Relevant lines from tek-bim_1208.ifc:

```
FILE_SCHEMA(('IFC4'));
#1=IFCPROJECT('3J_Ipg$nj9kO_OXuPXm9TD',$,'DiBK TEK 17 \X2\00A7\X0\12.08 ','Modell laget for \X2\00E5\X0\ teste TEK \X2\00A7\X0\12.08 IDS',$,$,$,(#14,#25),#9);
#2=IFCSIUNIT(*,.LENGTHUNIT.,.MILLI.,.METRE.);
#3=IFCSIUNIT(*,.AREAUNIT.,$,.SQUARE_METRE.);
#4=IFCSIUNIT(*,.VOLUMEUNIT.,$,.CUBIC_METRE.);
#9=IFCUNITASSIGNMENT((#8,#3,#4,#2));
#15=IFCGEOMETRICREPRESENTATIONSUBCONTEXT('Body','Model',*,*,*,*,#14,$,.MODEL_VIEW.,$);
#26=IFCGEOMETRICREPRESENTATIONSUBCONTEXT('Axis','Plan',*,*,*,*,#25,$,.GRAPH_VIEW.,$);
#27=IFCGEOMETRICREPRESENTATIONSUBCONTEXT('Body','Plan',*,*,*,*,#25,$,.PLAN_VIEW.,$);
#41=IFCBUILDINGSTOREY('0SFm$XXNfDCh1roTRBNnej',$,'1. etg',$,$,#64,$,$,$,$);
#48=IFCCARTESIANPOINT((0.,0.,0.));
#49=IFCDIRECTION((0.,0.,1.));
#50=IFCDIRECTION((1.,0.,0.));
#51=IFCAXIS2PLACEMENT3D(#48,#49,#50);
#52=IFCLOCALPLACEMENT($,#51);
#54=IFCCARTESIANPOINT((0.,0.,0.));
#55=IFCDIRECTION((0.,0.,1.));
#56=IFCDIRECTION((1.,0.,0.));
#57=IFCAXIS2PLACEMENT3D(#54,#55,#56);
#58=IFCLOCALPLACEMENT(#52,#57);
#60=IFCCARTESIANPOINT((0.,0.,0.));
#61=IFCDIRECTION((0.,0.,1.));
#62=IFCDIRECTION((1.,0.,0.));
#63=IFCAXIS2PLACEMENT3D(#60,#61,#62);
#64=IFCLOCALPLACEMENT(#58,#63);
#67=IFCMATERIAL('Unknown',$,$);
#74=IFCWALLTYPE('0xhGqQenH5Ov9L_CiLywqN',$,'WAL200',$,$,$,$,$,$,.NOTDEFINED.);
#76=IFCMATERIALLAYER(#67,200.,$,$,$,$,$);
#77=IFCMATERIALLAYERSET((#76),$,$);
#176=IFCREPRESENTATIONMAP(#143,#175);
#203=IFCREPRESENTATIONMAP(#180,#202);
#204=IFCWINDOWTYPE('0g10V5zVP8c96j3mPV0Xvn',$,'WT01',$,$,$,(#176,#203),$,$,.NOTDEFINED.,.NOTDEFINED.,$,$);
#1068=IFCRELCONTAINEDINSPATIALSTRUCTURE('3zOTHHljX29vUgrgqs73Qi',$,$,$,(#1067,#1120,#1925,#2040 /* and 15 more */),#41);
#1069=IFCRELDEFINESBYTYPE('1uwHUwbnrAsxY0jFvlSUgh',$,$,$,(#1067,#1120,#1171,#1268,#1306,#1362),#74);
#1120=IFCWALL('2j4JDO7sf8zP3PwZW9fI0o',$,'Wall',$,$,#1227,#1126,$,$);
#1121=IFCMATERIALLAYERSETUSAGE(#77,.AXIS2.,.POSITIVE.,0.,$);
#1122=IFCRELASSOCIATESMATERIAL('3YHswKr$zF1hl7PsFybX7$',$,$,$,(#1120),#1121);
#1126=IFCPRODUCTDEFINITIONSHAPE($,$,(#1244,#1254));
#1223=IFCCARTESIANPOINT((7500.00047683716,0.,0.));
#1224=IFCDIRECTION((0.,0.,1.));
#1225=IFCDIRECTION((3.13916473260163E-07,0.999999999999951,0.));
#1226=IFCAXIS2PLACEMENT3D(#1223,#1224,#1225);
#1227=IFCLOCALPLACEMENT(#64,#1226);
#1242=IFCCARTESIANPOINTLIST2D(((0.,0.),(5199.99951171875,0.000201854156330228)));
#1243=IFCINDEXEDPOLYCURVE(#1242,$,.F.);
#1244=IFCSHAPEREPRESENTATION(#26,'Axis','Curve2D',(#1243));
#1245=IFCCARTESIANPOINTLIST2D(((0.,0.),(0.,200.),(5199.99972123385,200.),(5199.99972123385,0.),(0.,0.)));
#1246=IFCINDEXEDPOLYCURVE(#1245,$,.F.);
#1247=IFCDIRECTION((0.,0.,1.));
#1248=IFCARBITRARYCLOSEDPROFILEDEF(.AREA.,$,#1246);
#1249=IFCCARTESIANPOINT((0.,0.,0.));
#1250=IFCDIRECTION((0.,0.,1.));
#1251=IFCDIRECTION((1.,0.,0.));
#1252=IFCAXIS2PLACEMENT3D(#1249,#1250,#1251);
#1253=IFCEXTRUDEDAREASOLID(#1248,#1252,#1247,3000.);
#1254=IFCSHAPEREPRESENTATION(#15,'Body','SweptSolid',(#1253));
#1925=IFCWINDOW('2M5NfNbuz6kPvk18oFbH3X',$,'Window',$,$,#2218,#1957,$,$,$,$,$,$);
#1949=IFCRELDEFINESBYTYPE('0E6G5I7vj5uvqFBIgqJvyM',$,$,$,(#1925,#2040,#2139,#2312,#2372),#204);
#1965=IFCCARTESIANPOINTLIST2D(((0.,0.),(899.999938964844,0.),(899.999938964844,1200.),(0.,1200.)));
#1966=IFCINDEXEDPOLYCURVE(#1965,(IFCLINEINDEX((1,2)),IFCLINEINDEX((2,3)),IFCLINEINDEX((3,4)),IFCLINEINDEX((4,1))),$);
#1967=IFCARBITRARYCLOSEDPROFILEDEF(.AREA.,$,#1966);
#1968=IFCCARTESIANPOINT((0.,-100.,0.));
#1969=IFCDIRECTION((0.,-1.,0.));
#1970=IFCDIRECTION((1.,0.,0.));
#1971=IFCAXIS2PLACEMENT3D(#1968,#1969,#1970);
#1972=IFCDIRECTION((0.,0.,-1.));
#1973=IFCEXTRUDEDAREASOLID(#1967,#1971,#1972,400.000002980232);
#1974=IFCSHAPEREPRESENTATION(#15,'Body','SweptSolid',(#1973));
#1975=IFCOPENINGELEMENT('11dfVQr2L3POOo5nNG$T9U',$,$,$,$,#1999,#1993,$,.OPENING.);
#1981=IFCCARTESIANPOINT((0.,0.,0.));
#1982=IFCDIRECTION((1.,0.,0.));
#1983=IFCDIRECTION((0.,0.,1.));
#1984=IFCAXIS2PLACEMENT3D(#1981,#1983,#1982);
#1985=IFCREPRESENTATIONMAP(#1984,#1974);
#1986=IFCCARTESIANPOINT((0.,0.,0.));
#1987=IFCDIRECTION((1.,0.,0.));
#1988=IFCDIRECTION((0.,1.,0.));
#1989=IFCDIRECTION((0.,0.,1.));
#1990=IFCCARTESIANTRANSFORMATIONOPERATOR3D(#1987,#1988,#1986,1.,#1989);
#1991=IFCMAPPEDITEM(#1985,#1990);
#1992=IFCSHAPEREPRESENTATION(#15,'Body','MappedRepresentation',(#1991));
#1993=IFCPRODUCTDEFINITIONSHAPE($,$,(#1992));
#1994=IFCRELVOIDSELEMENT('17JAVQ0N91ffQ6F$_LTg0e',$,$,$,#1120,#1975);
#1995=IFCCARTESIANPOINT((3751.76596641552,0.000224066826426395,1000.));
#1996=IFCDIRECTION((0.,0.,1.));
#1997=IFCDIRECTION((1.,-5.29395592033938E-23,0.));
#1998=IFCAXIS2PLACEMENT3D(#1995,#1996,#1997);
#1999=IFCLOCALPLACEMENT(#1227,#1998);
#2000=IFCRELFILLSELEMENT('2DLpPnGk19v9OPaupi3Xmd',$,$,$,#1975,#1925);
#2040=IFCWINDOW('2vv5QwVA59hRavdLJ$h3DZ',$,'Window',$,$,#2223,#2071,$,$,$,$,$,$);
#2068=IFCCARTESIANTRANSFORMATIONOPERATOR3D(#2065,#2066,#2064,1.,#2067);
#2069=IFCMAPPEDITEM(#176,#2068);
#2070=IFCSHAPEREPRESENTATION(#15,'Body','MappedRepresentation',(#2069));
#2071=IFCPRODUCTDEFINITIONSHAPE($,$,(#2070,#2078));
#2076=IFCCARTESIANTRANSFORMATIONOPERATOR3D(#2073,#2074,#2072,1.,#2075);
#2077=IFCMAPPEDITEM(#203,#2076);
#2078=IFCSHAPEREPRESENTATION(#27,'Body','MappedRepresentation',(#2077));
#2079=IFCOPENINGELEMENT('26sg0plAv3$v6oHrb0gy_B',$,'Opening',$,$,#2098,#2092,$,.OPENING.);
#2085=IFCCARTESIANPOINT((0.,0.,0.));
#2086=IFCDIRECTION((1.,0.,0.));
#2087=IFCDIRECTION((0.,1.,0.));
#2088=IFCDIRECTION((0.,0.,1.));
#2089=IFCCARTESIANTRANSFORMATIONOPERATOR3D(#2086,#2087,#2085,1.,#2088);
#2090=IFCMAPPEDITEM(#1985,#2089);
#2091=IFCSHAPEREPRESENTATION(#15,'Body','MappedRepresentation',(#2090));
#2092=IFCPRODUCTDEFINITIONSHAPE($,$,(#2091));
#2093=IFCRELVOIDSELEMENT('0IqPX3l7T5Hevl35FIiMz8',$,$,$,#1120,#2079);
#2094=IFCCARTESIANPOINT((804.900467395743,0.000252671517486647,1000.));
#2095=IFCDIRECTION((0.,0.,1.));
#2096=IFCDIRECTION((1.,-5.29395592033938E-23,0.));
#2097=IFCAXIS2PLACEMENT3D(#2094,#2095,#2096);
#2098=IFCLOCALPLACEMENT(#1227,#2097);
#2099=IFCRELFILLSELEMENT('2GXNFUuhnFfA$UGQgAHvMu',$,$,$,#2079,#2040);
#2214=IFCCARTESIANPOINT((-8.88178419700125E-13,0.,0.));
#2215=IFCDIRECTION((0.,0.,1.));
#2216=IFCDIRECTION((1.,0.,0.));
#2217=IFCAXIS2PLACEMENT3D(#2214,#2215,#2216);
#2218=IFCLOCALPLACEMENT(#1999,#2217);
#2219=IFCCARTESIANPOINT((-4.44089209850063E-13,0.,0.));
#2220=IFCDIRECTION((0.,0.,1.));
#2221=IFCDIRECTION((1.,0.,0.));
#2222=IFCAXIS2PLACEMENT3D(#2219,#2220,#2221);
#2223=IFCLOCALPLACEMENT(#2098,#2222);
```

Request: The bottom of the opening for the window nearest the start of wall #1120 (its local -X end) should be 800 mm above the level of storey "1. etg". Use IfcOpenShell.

```python
import numpy as np
import ifcopenshell
import ifcopenshell.api.geometry
import ifcopenshell.geom
import ifcopenshell.util.element
import ifcopenshell.util.placement
import ifcopenshell.util.shape
import ifcopenshell.util.unit

model = ifcopenshell.open("tek-bim_1208.ifc")
unit_scale = ifcopenshell.util.unit.calculate_unit_scale(model)

window = model.by_id(2040)
opening = window.FillsVoids[0].RelatingOpeningElement
storey = ifcopenshell.util.element.get_container(window, ifc_class="IfcBuildingStorey")
level = ifcopenshell.util.placement.get_local_placement(storey.ObjectPlacement)[2, 3]

# The opening's origin need not be at the sill, so measure its lowest point.
shape = ifcopenshell.geom.create_shape(ifcopenshell.geom.settings(), opening)
bottom = ifcopenshell.util.shape.get_shape_bottom_elevation(shape, shape.geometry) / unit_scale
dz = level + 0.8 / unit_scale - bottom

shift = np.array([0.0, 0.0, dz])
# The window is placed relative to its opening, so it follows when the opening moves.
matrix = ifcopenshell.util.placement.get_local_placement(opening.ObjectPlacement)
matrix[:3, 3] += shift
ifcopenshell.api.geometry.edit_object_placement(
    model, product=opening, matrix=matrix, is_si=False, should_transform_children=True
)

print(f"moved by {dz * unit_scale:+.3f} m")

model.write("tek-bim_1208_edited.ifc")
```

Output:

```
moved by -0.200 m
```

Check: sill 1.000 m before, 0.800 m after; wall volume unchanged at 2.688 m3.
